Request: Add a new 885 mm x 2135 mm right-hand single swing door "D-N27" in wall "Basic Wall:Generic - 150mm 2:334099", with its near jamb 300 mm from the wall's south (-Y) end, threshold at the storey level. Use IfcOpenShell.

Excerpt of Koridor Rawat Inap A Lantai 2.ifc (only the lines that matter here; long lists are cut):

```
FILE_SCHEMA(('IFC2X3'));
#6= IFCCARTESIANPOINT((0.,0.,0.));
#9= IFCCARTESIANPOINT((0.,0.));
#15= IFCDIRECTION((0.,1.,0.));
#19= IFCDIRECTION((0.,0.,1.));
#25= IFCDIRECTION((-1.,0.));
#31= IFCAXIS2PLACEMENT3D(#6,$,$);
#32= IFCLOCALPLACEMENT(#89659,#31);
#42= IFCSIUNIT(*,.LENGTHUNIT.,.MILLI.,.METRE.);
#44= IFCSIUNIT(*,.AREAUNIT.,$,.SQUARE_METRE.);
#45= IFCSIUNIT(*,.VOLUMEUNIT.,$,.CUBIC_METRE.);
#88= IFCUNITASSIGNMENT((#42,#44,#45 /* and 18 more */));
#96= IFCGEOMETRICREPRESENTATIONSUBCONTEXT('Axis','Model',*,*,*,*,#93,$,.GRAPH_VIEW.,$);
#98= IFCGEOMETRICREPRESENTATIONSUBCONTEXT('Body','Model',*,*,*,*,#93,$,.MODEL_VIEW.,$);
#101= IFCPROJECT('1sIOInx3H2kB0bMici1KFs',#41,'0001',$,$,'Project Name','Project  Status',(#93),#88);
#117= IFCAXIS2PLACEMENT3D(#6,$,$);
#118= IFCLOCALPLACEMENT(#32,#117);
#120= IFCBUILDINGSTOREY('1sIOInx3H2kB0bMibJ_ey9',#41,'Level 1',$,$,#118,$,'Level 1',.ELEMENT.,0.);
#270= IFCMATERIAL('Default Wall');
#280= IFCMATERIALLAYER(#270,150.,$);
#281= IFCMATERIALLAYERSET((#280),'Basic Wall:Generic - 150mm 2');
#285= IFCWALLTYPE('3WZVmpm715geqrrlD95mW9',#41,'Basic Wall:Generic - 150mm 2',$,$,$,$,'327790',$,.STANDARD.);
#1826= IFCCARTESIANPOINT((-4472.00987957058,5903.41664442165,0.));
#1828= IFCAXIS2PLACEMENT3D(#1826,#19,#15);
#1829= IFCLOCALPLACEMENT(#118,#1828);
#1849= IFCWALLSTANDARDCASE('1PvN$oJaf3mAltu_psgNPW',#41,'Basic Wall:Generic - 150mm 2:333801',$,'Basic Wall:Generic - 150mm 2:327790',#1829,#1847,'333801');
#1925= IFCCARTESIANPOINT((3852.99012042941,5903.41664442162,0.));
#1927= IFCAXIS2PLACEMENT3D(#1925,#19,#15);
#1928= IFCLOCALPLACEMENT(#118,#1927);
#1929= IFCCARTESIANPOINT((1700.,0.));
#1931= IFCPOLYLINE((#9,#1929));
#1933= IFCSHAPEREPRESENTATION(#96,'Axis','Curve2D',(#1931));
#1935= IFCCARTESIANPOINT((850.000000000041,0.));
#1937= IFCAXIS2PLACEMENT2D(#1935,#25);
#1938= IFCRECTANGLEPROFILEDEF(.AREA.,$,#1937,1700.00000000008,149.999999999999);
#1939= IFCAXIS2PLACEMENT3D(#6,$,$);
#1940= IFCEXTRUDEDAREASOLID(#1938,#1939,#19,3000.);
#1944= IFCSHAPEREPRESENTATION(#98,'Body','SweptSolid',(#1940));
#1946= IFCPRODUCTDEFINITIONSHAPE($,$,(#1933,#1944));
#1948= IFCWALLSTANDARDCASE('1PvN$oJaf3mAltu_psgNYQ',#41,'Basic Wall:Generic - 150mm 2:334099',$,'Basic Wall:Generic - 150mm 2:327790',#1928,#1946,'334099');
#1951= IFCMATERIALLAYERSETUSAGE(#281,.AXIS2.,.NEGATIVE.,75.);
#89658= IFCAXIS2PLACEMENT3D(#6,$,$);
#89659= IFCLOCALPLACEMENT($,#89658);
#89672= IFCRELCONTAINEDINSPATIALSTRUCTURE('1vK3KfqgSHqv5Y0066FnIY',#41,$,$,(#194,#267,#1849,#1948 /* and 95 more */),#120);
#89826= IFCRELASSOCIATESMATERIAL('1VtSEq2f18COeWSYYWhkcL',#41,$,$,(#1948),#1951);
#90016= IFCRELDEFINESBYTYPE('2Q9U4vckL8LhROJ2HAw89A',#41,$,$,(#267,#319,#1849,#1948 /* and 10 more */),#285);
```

```python
import numpy as np
import ifcopenshell
import ifcopenshell.api.feature
import ifcopenshell.api.geometry
import ifcopenshell.api.root
import ifcopenshell.api.spatial
import ifcopenshell.api.type
import ifcopenshell.geom
import ifcopenshell.util.element
import ifcopenshell.util.placement
import ifcopenshell.util.representation
import ifcopenshell.util.shape
import ifcopenshell.util.unit

model = ifcopenshell.open("Koridor Rawat Inap A Lantai 2.ifc")
unit_scale = ifcopenshell.util.unit.calculate_unit_scale(model)
settings = ifcopenshell.geom.settings()


def volume(element):
    """Net volume in cubic metres, openings subtracted."""
    shape = ifcopenshell.geom.create_shape(settings, element)
    return ifcopenshell.util.shape.get_volume(shape.geometry)


wall = model.by_guid("1PvN$oJaf3mAltu_psgNYQ")
storey = ifcopenshell.util.element.get_container(wall, ifc_class="IfcBuildingStorey")
context = ifcopenshell.util.representation.get_context(model, "Model", "Body", "MODEL_VIEW")
before = volume(wall)

width, height, from_end, sill = 0.885, 2.135, 0.3, 0.0  # metres

# The wall runs along its own X axis, and the end named is its -X end.
wall_shape = ifcopenshell.geom.create_shape(settings, wall)
x, y, z = ifcopenshell.util.shape.get_vertices(wall_shape.geometry).T
start = x.min() + from_end
face, thickness = float(y.min()), float(y.max() - y.min())
wall_matrix = ifcopenshell.util.placement.get_local_placement(wall.ObjectPlacement)
level = ifcopenshell.util.placement.get_local_placement(storey.ObjectPlacement)[2, 3]


def in_wall(x, y):
    """Placement at x, y metres in the wall's axes, at sill height."""
    matrix = wall_matrix.copy()
    matrix[:, 3] = wall_matrix @ np.array([x / unit_scale, y / unit_scale, 0.0, 1.0])
    matrix[2, 3] = level + sill / unit_scale
    return matrix


# Opening: a box that overshoots both wall faces by 50 mm.
opening = ifcopenshell.api.root.create_entity(model, ifc_class="IfcOpeningElement")
box = ifcopenshell.api.geometry.add_wall_representation(
    model, context=context, length=width, height=height, thickness=thickness + 0.1
)
ifcopenshell.api.geometry.assign_representation(model, product=opening, representation=box)
ifcopenshell.api.geometry.edit_object_placement(model, product=opening, matrix=in_wall(start, face - 0.05), is_si=False)
ifcopenshell.api.feature.add_feature(model, feature=opening, element=wall)

door = ifcopenshell.api.root.create_entity(model, ifc_class="IfcDoor", name="D-N27")
door.OverallWidth, door.OverallHeight = width / unit_scale, height / unit_scale
body = ifcopenshell.api.geometry.add_door_representation(
    model,
    context=context,
    overall_width=door.OverallWidth,
    overall_height=door.OverallHeight,
    operation_type="SINGLE_SWING_RIGHT",
    lining_properties={"LiningDepth": thickness / unit_scale, "ThresholdDepth": thickness / unit_scale},
)
ifcopenshell.api.geometry.assign_representation(model, product=door, representation=body)
ifcopenshell.api.spatial.assign_container(model, products=[door], relating_structure=storey)
fills = ifcopenshell.api.feature.add_filling(model, opening=opening, element=door)
fills.OwnerHistory = door.OwnerHistory  # required in IFC2X3

# IFC2X3 keeps the operation on the door style.
style = ifcopenshell.api.root.create_entity(model, ifc_class="IfcDoorStyle", name="D-N27")
style.OperationType, style.ConstructionType = "SINGLE_SWING_RIGHT", "NOTDEFINED"
style.ParameterTakesPrecedence = style.Sizeable = False
ifcopenshell.api.type.assign_type(model, related_objects=[door], relating_type=style)

# The lining spans the wall, so the door starts at the wall face.
ifcopenshell.api.geometry.edit_object_placement(model, product=door, matrix=in_wall(start, face), is_si=False)

after = volume(wall)

print(f"wall volume {before:.3f} -> {after:.3f} m3")

model.write("Koridor Rawat Inap A Lantai 2_updated.ifc")
```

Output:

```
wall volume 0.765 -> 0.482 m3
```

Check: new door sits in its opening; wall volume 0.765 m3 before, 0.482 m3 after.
